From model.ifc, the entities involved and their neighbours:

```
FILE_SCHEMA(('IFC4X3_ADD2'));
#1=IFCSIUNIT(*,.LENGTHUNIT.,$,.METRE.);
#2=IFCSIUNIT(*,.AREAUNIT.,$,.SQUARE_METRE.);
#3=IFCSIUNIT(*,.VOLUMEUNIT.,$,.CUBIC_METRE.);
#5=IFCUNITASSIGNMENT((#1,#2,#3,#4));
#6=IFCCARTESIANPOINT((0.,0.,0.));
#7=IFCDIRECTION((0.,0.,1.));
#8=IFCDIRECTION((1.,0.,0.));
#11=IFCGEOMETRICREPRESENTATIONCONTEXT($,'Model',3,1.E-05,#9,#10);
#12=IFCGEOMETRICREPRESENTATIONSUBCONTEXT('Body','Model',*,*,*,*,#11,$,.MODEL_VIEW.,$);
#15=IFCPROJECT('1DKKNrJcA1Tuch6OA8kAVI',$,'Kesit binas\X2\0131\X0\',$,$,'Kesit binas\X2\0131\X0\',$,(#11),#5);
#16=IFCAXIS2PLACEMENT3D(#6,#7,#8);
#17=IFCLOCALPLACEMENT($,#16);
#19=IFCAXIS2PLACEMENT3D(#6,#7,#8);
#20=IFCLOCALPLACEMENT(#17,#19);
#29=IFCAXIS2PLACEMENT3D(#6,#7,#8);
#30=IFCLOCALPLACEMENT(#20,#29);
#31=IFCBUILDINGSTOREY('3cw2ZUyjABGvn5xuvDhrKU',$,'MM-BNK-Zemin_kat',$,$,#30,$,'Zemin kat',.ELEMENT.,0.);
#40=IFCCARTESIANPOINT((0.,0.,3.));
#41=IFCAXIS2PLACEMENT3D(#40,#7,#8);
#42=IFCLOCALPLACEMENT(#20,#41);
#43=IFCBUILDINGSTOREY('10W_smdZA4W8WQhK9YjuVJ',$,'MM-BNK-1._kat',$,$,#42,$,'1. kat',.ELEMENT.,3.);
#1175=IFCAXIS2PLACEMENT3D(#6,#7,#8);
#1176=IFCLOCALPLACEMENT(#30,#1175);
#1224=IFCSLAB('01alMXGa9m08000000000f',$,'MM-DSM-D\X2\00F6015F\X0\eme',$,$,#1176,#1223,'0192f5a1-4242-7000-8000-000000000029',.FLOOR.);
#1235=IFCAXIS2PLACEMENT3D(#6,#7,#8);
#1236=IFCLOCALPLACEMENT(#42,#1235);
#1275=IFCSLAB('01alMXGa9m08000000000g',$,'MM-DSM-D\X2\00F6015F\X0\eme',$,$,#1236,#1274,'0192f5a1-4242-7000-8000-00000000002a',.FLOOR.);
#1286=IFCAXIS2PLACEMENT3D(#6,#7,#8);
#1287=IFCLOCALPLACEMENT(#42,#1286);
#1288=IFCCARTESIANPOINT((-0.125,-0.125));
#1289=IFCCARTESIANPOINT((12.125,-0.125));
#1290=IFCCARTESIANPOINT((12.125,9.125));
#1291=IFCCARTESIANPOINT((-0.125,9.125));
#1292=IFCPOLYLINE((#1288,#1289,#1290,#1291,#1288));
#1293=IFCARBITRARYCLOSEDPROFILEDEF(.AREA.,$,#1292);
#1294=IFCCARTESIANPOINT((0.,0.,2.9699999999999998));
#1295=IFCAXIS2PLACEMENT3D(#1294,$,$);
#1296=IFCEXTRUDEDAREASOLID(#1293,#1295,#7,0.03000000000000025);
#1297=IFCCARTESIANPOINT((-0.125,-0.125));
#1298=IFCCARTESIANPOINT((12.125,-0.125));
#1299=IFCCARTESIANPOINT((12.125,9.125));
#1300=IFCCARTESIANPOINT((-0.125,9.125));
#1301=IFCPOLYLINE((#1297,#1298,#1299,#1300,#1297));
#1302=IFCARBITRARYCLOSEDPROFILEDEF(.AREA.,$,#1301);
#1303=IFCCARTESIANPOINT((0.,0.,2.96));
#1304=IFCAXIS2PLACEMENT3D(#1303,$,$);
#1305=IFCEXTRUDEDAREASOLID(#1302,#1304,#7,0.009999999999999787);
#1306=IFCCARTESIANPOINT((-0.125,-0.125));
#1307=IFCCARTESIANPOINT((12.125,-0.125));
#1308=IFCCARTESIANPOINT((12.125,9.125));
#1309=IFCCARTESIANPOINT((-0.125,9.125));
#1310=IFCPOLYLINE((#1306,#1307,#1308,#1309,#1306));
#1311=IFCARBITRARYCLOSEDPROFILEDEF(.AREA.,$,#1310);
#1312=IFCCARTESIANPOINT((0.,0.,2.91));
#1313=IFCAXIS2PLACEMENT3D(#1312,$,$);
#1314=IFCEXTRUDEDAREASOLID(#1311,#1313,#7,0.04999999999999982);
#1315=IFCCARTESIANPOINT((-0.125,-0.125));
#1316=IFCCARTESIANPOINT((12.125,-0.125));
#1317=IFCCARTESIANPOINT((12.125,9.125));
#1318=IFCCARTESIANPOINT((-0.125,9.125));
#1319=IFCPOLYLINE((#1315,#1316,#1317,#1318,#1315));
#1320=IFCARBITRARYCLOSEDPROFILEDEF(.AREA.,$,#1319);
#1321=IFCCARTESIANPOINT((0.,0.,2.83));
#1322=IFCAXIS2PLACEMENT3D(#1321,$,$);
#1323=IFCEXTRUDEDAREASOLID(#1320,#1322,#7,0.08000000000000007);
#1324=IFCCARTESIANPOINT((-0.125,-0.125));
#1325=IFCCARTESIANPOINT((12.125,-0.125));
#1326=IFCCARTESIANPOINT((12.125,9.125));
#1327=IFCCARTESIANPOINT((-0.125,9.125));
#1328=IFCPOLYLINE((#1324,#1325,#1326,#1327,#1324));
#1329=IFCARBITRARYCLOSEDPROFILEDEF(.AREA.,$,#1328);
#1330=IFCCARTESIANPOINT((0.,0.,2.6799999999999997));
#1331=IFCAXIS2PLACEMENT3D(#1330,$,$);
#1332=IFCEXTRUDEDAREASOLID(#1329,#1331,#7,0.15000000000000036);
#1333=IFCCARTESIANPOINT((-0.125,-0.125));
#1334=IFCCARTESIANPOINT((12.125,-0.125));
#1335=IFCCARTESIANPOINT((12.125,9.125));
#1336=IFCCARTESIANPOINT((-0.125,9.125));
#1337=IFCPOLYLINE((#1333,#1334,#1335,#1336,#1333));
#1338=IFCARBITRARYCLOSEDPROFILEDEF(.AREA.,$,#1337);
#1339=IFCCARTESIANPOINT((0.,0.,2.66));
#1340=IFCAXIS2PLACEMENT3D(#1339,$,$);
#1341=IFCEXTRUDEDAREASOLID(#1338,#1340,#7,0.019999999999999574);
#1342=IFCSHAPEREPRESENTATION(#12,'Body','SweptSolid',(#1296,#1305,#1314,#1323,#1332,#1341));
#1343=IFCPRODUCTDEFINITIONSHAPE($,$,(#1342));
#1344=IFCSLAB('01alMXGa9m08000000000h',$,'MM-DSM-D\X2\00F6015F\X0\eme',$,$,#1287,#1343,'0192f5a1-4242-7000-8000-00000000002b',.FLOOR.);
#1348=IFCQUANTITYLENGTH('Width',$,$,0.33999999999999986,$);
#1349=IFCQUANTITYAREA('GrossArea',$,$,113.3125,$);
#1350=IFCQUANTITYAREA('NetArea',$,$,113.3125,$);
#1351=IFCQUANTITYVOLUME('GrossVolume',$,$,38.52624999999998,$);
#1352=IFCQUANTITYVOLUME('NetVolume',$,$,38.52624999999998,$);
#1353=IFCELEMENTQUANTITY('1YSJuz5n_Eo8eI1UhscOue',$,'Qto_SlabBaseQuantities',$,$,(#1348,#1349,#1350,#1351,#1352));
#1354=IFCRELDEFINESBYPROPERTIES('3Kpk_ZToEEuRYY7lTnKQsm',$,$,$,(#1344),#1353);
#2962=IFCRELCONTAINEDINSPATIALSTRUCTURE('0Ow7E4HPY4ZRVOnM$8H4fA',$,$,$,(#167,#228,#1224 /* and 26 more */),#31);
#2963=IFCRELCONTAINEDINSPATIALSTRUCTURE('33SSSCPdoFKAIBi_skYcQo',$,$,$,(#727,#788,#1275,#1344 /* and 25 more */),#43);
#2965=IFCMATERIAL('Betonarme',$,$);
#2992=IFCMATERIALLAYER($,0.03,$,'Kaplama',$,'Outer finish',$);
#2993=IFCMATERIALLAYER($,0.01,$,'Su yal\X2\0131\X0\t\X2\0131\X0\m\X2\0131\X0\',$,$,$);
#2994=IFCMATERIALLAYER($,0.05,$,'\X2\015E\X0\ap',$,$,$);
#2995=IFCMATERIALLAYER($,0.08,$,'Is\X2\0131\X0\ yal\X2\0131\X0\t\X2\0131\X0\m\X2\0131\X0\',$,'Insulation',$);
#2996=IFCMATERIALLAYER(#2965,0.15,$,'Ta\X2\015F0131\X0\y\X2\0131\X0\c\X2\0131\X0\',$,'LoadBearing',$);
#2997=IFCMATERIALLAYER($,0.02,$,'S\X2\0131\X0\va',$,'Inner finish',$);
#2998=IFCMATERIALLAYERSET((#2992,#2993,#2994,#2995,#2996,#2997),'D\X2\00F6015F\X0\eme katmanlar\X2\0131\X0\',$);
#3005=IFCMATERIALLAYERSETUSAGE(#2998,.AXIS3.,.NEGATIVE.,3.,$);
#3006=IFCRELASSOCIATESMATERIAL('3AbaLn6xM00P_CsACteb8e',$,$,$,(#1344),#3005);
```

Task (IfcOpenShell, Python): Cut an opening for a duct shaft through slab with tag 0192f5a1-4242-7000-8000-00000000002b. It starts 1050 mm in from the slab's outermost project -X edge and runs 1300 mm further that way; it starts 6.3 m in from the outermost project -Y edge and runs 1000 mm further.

```python
import numpy as np
import ifcopenshell
import ifcopenshell.api.feature
import ifcopenshell.api.geometry
import ifcopenshell.api.pset
import ifcopenshell.api.root
import ifcopenshell.geom
import ifcopenshell.util.element
import ifcopenshell.util.placement
import ifcopenshell.util.representation
import ifcopenshell.util.shape
import ifcopenshell.util.unit

model = ifcopenshell.open("model.ifc")
unit_scale = ifcopenshell.util.unit.calculate_unit_scale(model)
area_scale = ifcopenshell.util.unit.calculate_unit_scale(model, "AREAUNIT")
volume_scale = ifcopenshell.util.unit.calculate_unit_scale(model, "VOLUMEUNIT")
settings = ifcopenshell.geom.settings()


def volume(element):
    """Net volume in cubic metres, openings subtracted."""
    shape = ifcopenshell.geom.create_shape(settings, element)
    return ifcopenshell.util.shape.get_volume(shape.geometry)


slab = model.by_guid("01alMXGa9m08000000000h")
before = volume(slab)

# Extent in the slab's own axes, in metres. The edges named are its -X and -Y sides.
slab_shape = ifcopenshell.geom.create_shape(settings, slab)
vertices = ifcopenshell.util.shape.get_vertices(slab_shape.geometry)
x_min, y_min, bottom = vertices.min(axis=0)
top = vertices[:, 2].max()

opening = ifcopenshell.api.root.create_entity(model, ifc_class="IfcOpeningElement", name="Duct shaft opening", predefined_type="OPENING")
context = ifcopenshell.util.representation.get_context(model, "Model", "Body", "MODEL_VIEW")
width, depth = 1.3, 1
outline = [(0.0, 0.0), (width, 0.0), (width, depth), (0.0, depth), (0.0, 0.0)]
# Overshoot both faces by 50 mm so the cut is clean.
shape = ifcopenshell.api.geometry.add_slab_representation(
    model, context=context, depth=top - bottom + 0.1, polyline=outline
)
ifcopenshell.api.geometry.assign_representation(model, product=opening, representation=shape)

matrix = ifcopenshell.util.placement.get_local_placement(slab.ObjectPlacement)
matrix[:, 3] = matrix @ np.append(np.array([x_min + 1.05, y_min + 6.3, bottom - 0.05]) / unit_scale, 1.0)
ifcopenshell.api.geometry.edit_object_placement(model, product=opening, matrix=matrix, is_si=False)
ifcopenshell.api.feature.add_feature(model, feature=opening, element=slab)

after = volume(slab)

# Update the slab's stored quantities.
qto = model.by_id(ifcopenshell.util.element.get_pset(slab, "Qto_SlabBaseQuantities", should_inherit=False)["id"])
ifcopenshell.api.pset.edit_qto(model, qto=qto, properties={
    "NetArea": after / (top - bottom) / area_scale,
    "NetVolume": after / volume_scale,
})

print(f"slab volume {before:.3f} -> {after:.3f} m3")

model.write("model_rev.ifc")
```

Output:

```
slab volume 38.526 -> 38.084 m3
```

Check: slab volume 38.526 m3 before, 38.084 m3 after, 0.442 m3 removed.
